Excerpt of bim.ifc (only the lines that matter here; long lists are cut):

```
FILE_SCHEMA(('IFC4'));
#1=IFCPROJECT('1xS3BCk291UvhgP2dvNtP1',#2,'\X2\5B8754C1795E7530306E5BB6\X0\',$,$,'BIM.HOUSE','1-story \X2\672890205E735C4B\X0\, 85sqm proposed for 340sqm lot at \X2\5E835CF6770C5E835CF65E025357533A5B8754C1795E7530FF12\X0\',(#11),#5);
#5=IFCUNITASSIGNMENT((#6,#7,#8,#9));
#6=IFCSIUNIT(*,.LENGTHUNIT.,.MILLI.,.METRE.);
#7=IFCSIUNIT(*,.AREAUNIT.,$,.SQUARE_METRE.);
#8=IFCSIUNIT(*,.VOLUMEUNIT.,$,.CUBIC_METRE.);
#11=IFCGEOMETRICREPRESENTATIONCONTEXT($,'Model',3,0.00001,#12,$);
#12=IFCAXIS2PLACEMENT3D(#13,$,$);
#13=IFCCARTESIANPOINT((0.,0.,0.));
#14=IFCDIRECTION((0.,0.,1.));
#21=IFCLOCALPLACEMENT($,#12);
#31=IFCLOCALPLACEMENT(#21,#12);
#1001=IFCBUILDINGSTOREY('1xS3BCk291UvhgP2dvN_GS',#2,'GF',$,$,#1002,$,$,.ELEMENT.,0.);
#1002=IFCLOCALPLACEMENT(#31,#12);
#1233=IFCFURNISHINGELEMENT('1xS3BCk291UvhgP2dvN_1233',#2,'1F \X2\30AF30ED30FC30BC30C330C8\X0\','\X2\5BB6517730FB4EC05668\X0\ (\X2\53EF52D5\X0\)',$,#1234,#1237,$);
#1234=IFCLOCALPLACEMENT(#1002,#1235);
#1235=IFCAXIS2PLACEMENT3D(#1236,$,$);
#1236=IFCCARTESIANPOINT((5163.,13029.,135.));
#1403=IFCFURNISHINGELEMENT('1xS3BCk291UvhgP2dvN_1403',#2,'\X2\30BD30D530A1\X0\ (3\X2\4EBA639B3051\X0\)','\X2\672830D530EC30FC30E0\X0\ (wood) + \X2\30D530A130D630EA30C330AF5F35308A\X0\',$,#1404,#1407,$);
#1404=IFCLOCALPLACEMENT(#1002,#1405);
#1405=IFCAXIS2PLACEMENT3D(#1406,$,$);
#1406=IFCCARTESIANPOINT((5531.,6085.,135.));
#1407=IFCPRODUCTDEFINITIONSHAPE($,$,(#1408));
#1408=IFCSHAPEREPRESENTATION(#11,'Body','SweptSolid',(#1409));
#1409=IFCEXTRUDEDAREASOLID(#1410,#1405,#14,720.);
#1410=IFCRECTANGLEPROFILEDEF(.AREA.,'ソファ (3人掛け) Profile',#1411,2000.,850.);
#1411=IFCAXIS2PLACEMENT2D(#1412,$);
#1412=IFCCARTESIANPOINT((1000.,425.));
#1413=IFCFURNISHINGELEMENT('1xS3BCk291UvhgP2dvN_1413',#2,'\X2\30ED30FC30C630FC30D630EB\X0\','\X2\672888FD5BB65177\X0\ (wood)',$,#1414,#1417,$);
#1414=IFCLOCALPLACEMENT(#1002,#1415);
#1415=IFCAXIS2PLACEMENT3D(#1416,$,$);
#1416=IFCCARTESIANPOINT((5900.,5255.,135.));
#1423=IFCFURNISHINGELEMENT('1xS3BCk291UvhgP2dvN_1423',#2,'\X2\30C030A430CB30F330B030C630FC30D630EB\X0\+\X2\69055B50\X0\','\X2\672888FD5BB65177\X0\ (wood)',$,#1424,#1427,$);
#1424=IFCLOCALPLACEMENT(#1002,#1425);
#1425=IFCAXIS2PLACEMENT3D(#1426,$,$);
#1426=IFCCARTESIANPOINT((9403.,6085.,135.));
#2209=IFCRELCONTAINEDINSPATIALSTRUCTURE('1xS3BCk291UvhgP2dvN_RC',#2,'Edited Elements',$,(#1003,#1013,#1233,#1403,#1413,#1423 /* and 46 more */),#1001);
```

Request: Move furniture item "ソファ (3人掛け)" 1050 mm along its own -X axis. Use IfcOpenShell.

```python
import ifcopenshell
import ifcopenshell.api.geometry
import ifcopenshell.util.placement
import ifcopenshell.util.unit

model = ifcopenshell.open("bim.ifc")
unit_scale = ifcopenshell.util.unit.calculate_unit_scale(model)

item = model.by_guid("1xS3BCk291UvhgP2dvN_1403")
matrix = ifcopenshell.util.placement.get_local_placement(item.ObjectPlacement)
matrix[:3, 3] -= matrix[:3, 0] * 1.05 / unit_scale
ifcopenshell.api.geometry.edit_object_placement(model, product=item, matrix=matrix, is_si=False)

print(ifcopenshell.util.placement.get_local_placement(item.ObjectPlacement).round(3) + 0.0)

model.write("bim_updated.ifc")
```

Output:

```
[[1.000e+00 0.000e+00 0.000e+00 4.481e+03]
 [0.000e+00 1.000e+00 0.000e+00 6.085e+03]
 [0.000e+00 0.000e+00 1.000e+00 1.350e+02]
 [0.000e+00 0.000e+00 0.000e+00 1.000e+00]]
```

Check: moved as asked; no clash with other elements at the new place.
